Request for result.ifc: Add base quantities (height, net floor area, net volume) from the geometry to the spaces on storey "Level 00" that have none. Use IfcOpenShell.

First a look at what the model holds.

```python
import ifcopenshell
import ifcopenshell.util.element
import ifcopenshell.util.unit

model = ifcopenshell.open("result.ifc")
print(model.schema)
for unit_type in ("LENGTHUNIT", "AREAUNIT", "VOLUMEUNIT"):
    print(unit_type, ifcopenshell.util.unit.calculate_unit_scale(model, unit_type))
storey = next(s for s in model.by_type("IfcBuildingStorey") if s.Name == "Level 00")
spaces = [e for e in ifcopenshell.util.element.get_decomposition(storey) if e.is_a("IfcSpace")]
for e in sorted(spaces, key=lambda e: e.id()):
    print(e.id(), e.is_a(), e.Name, list(ifcopenshell.util.element.get_psets(e, qtos_only=True)), sep=" | ")
```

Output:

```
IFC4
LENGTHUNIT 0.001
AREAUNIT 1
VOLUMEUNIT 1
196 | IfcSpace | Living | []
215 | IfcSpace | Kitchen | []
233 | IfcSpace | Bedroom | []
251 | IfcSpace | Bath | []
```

```python
import ifcopenshell
import ifcopenshell.api.pset
import ifcopenshell.geom
import ifcopenshell.util.element
import ifcopenshell.util.shape
import ifcopenshell.util.unit

model = ifcopenshell.open("result.ifc")
unit_scale = ifcopenshell.util.unit.calculate_unit_scale(model)
area_scale = ifcopenshell.util.unit.calculate_unit_scale(model, "AREAUNIT")
volume_scale = ifcopenshell.util.unit.calculate_unit_scale(model, "VOLUMEUNIT")
settings = ifcopenshell.geom.settings()

storey = next(s for s in model.by_type("IfcBuildingStorey") if s.Name == "Level 00")
spaces = [e for e in ifcopenshell.util.element.get_decomposition(storey) if e.is_a("IfcSpace")]

for e in sorted(spaces, key=lambda e: e.id()):
    if ifcopenshell.util.element.get_psets(e, qtos_only=True, should_inherit=False):
        continue
    # Geometry comes back in metres, in the element's own axes.
    shape = ifcopenshell.geom.create_shape(settings, e)
    values = {
        "Height": ifcopenshell.util.shape.get_z(shape.geometry) / unit_scale,
        "NetFloorArea": ifcopenshell.util.shape.get_footprint_area(shape.geometry) / area_scale,
        "NetVolume": ifcopenshell.util.shape.get_volume(shape.geometry) / volume_scale,
    }
    qto = ifcopenshell.api.pset.add_qto(model, product=e, name="Qto_SpaceBaseQuantities")
    ifcopenshell.api.pset.edit_qto(model, qto=qto, properties=values)
    print(e.id(), {k: round(v, 3) for k, v in values.items()})

model.write("result_v2.ifc")
```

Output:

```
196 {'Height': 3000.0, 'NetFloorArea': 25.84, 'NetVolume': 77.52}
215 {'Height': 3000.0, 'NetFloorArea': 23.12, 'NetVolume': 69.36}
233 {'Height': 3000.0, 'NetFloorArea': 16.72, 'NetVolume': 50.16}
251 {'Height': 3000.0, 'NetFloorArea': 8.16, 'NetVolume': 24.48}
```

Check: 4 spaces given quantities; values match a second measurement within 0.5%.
